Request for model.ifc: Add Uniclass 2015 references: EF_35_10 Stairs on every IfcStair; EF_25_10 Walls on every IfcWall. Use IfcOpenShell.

First a look at what the model holds.

```python
import ifcopenshell

model = ifcopenshell.open("model.ifc")
print(model.schema)
print("classifications:", [c.Name for c in model.by_type("IfcClassification")])
for ifc_class in ("IfcDoor", "IfcRoof", "IfcStair", "IfcWall", "IfcWindow"):
    print(ifc_class, len(model.by_type(ifc_class)))
```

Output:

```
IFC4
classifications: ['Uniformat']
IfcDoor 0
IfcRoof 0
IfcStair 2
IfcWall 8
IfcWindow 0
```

```python
import ifcopenshell
import ifcopenshell.api.classification

model = ifcopenshell.open("model.ifc")

system = ifcopenshell.api.classification.add_classification(model, classification="Uniclass 2015")

codes = {
    "IfcStair": ("EF_35_10", "Stairs"),
    "IfcWall": ("EF_25_10", "Walls"),
}
for ifc_class, (code, name) in codes.items():
    products = model.by_type(ifc_class)
    ifcopenshell.api.classification.add_reference(
        model, products=products, classification=system, identification=code, name=name
    )
    print(code, len(products))

model.write("model_rev.ifc")
```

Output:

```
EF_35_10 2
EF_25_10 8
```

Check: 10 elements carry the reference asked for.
